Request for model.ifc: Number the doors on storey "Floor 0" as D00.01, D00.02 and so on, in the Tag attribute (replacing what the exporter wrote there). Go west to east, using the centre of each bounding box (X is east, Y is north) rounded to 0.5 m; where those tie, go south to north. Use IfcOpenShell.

First a look at what the model holds.

```python
import ifcopenshell
import ifcopenshell.util.element
import ifcopenshell.util.placement

model = ifcopenshell.open("model.ifc")
print(model.schema)
storey = next(s for s in model.by_type("IfcBuildingStorey") if s.Name == "Floor 0")
doors = [e for e in ifcopenshell.util.element.get_decomposition(storey) if e.is_a("IfcDoor")]
for e in sorted(doors, key=lambda e: e.id()):
    origin = ifcopenshell.util.placement.get_local_placement(e.ObjectPlacement)[:3, 3]
    print(e.id(), e.Tag, e.Name, origin.round(2) + 0.0, sep=" | ")
```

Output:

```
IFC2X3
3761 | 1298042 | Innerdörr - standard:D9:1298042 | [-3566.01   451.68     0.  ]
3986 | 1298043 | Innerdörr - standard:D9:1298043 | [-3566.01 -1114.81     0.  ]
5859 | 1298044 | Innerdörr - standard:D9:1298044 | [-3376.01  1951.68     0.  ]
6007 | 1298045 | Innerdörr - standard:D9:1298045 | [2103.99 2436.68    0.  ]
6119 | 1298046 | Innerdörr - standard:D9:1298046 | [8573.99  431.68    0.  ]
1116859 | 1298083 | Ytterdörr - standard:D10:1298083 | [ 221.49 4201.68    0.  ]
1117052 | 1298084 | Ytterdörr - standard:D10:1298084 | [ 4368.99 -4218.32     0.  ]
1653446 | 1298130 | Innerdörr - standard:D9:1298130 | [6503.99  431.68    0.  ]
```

```python
import ifcopenshell
import ifcopenshell.geom
import ifcopenshell.util.element
import ifcopenshell.util.shape

model = ifcopenshell.open("model.ifc")
settings = ifcopenshell.geom.settings()
settings.set("use-world-coords", True)


def centre(element):
    shape = ifcopenshell.geom.create_shape(settings, element)
    return ifcopenshell.util.shape.get_bbox_centroid(shape.geometry)


storey = next(s for s in model.by_type("IfcBuildingStorey") if s.Name == "Floor 0")
doors = [e for e in ifcopenshell.util.element.get_decomposition(storey) if e.is_a("IfcDoor")]

# Insertion points can sit at a corner or the storey origin, so sort by the geometry (in metres).
centres = {e: centre(e) for e in doors}
doors.sort(key=lambda e: (round(centres[e][0] / 0.5), centres[e][1]))

for i, e in enumerate(doors, start=1):
    number = f"D00.{i:02d}"
    e.Tag = number
    print(e.id(), number)

model.write("model_rev.ifc")
```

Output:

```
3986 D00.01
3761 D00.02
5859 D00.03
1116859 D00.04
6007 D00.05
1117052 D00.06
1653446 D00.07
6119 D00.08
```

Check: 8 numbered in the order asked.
